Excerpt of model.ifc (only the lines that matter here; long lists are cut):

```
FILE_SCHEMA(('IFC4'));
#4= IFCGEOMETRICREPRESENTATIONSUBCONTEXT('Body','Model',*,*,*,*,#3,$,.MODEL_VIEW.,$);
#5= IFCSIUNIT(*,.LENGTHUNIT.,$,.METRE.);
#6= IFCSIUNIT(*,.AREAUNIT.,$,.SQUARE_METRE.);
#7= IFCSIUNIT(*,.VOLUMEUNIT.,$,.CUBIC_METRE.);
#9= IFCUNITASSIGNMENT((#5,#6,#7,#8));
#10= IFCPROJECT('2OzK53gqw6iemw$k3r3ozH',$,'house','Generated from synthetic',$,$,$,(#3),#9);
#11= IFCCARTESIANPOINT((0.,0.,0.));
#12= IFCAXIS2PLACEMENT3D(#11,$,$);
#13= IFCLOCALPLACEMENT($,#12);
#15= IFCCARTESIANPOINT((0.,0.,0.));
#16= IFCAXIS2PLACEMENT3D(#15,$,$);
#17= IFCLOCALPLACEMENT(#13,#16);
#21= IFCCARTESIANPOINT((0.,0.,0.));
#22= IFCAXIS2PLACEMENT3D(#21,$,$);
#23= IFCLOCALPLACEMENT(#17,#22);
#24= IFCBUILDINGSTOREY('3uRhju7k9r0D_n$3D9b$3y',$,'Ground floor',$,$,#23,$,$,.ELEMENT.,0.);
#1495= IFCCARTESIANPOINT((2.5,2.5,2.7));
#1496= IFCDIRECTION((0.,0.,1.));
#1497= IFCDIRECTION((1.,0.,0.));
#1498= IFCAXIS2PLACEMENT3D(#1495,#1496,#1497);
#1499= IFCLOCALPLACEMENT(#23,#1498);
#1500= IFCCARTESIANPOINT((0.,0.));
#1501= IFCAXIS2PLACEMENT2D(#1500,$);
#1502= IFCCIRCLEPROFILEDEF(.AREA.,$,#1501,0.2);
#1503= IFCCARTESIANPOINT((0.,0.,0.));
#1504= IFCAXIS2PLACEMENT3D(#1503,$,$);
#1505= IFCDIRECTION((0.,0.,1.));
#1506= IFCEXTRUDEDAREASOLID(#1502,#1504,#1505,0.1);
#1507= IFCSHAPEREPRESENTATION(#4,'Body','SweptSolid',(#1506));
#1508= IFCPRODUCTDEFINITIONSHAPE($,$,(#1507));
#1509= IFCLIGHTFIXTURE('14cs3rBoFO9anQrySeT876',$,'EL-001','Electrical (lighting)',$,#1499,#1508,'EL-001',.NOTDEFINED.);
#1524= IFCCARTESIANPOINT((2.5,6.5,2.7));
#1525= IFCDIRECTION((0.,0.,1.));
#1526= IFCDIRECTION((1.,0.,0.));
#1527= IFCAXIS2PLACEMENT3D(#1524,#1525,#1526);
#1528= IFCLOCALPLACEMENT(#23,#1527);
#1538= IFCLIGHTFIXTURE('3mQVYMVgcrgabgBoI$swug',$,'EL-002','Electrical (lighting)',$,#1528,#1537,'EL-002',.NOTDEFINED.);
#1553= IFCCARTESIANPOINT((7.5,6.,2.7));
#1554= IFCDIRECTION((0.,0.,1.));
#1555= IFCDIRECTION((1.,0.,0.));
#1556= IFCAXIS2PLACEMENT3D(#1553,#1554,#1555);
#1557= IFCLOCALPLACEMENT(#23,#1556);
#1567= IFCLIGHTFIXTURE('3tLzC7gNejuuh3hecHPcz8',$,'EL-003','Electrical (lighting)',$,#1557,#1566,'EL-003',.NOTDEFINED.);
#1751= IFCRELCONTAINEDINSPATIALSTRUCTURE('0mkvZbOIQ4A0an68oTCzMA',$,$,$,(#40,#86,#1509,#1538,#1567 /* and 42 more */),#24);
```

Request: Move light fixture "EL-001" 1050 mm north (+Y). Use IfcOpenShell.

```python
import ifcopenshell
import ifcopenshell.api.geometry
import ifcopenshell.util.placement
import ifcopenshell.util.unit

model = ifcopenshell.open("model.ifc")
unit_scale = ifcopenshell.util.unit.calculate_unit_scale(model)

item = model.by_guid("14cs3rBoFO9anQrySeT876")
matrix = ifcopenshell.util.placement.get_local_placement(item.ObjectPlacement)
matrix[1, 3] += 1.05 / unit_scale
ifcopenshell.api.geometry.edit_object_placement(model, product=item, matrix=matrix, is_si=False)

print(ifcopenshell.util.placement.get_local_placement(item.ObjectPlacement).round(3) + 0.0)

model.write("model_v2.ifc")
```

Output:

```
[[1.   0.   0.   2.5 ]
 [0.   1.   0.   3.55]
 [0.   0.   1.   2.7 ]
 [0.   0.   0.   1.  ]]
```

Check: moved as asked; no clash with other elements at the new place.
